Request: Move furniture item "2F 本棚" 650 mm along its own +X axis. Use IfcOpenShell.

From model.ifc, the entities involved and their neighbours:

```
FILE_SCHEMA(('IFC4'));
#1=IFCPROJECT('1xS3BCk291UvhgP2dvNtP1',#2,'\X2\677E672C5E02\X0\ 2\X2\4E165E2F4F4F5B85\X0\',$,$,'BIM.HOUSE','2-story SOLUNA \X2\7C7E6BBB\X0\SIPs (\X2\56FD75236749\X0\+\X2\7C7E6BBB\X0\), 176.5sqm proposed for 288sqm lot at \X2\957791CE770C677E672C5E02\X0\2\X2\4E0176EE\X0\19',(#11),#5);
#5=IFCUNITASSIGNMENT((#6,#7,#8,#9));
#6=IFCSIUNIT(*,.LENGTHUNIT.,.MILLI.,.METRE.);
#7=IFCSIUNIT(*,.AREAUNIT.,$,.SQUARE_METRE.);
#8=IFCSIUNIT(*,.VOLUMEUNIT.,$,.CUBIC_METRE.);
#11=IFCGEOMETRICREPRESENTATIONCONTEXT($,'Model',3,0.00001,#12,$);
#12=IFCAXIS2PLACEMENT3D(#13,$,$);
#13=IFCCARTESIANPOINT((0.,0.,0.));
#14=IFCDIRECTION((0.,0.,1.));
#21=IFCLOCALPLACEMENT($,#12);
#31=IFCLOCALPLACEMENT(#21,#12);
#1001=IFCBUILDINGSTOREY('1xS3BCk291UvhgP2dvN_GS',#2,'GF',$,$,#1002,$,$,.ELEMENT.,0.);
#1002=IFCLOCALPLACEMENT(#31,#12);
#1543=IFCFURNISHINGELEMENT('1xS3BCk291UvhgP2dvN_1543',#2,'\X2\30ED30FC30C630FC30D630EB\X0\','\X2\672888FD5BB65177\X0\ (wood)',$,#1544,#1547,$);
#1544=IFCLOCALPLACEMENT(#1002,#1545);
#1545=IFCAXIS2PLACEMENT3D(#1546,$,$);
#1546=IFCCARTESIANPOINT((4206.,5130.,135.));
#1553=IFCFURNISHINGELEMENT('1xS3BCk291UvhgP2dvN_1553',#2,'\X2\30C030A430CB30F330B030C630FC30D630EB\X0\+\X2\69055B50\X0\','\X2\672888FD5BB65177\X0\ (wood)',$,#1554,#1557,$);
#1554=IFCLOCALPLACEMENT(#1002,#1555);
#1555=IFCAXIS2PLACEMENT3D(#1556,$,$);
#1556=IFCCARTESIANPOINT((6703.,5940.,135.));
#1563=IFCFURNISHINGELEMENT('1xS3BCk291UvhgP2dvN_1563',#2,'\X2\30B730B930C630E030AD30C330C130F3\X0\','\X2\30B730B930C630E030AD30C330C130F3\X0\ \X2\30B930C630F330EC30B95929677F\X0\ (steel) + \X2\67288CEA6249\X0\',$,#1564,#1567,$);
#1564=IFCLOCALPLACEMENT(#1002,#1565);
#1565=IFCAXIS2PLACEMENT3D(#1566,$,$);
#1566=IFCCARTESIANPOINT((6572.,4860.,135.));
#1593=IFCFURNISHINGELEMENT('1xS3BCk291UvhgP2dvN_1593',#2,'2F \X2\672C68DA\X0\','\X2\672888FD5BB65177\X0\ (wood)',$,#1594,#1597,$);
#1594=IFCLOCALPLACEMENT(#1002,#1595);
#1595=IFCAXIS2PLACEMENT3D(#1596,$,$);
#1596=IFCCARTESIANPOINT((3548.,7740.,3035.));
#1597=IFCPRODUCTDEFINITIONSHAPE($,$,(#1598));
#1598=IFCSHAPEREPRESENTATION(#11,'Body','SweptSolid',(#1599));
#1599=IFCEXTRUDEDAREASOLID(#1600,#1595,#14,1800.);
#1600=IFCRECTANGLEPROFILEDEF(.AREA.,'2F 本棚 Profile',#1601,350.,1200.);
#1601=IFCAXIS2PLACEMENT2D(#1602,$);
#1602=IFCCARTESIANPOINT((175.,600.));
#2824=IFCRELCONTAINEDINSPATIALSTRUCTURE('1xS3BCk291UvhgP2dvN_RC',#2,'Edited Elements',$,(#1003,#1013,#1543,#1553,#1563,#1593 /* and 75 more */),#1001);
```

```python
import ifcopenshell
import ifcopenshell.api.geometry
import ifcopenshell.util.placement

model = ifcopenshell.open("model.ifc")

item = model.by_guid("1xS3BCk291UvhgP2dvN_1593")
matrix = ifcopenshell.util.placement.get_local_placement(item.ObjectPlacement)
matrix[:3, 3] += matrix[:3, 0] * 650.0
ifcopenshell.api.geometry.edit_object_placement(model, product=item, matrix=matrix, is_si=False)

print(ifcopenshell.util.placement.get_local_placement(item.ObjectPlacement).round(3) + 0.0)

model.write("model_updated.ifc")
```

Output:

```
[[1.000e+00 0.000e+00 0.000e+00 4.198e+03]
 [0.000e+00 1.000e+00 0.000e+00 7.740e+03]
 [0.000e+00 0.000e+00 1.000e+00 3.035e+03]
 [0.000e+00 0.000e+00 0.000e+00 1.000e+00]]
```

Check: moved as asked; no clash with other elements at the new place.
